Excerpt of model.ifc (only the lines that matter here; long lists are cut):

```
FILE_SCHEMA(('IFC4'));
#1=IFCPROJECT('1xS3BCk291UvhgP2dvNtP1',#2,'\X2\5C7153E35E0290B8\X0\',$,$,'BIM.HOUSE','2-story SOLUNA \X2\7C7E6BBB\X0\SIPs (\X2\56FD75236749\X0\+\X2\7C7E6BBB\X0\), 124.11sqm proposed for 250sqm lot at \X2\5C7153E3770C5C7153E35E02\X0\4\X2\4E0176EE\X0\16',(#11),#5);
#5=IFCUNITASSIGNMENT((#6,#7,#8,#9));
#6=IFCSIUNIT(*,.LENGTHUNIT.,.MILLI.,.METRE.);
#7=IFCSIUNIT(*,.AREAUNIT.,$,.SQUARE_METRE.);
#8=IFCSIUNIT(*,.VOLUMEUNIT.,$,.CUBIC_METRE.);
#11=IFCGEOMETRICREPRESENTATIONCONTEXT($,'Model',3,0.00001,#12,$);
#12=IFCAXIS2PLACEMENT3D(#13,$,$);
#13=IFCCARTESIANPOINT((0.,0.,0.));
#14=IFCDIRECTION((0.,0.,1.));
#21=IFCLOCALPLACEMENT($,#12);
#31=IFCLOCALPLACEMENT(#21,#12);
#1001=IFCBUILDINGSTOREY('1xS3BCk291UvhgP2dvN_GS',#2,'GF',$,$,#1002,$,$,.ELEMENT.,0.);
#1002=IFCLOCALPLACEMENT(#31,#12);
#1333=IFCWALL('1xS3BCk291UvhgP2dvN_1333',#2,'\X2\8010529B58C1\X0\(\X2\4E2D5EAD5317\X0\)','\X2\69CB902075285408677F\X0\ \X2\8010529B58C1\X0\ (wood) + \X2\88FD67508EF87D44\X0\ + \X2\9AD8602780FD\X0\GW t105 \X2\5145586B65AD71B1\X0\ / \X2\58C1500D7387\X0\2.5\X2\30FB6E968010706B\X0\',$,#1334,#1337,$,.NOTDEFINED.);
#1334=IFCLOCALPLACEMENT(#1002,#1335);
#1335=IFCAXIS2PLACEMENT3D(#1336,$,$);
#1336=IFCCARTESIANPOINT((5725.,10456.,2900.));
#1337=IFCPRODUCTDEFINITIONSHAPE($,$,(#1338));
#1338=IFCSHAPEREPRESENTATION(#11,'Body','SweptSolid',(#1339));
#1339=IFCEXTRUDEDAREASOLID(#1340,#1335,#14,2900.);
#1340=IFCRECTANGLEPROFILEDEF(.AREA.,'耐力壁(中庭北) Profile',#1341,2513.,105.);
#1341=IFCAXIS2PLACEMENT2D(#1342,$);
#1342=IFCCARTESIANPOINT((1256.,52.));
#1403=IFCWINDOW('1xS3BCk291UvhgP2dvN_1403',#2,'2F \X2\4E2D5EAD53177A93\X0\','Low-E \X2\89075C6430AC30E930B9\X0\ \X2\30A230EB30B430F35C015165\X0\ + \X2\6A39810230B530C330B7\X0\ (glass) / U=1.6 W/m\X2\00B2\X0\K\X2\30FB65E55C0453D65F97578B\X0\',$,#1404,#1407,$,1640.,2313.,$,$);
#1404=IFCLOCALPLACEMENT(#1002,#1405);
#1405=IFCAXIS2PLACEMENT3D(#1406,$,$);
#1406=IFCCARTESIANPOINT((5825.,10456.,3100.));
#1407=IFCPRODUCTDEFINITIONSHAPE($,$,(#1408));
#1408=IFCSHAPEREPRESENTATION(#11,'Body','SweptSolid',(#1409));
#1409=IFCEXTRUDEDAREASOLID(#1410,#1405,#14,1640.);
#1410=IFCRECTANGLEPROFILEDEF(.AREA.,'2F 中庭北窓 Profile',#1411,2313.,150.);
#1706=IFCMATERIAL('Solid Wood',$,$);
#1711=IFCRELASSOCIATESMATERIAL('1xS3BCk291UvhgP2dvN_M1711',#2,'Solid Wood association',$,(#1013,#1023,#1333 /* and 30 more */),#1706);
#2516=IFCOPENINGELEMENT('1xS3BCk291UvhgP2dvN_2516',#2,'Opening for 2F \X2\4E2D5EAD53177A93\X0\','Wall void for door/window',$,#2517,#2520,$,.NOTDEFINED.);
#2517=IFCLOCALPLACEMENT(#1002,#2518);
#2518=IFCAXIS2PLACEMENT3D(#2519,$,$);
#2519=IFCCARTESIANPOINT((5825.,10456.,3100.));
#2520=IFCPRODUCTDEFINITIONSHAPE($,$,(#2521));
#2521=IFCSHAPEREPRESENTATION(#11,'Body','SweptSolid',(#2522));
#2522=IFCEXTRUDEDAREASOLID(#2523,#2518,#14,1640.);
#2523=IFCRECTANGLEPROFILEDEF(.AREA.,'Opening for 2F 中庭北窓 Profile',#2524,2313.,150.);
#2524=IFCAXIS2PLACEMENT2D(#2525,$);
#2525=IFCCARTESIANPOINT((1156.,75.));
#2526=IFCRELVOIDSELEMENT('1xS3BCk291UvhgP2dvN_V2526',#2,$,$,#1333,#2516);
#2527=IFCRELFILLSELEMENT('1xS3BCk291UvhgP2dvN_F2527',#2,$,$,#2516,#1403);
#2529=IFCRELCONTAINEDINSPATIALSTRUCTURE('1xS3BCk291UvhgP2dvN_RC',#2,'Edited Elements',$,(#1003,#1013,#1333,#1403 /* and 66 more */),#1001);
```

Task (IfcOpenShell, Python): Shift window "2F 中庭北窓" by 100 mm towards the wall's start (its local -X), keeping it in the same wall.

```python
import ifcopenshell
import ifcopenshell.api.geometry
import ifcopenshell.util.placement

model = ifcopenshell.open("model.ifc")

window = model.by_guid("1xS3BCk291UvhgP2dvN_1403")
opening = window.FillsVoids[0].RelatingOpeningElement
wall = opening.VoidsElements[0].RelatingBuildingElement

wall_matrix = ifcopenshell.util.placement.get_local_placement(wall.ObjectPlacement)
shift = wall_matrix[:3, 0] * -100.0
before = ifcopenshell.util.placement.get_local_placement(window.ObjectPlacement)[:3, 3].copy()

# The window is not placed relative to its opening, so move both.
for product in (opening, window):
    matrix = ifcopenshell.util.placement.get_local_placement(product.ObjectPlacement)
    matrix[:3, 3] += shift
    ifcopenshell.api.geometry.edit_object_placement(model, product=product, matrix=matrix, is_si=False)

after = ifcopenshell.util.placement.get_local_placement(window.ObjectPlacement)[:3, 3]
print("window moved by", (after - before).round(3) + 0.0)

model.write("model_v2.ifc")
```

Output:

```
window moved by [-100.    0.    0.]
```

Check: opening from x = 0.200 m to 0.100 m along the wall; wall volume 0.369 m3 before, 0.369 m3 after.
